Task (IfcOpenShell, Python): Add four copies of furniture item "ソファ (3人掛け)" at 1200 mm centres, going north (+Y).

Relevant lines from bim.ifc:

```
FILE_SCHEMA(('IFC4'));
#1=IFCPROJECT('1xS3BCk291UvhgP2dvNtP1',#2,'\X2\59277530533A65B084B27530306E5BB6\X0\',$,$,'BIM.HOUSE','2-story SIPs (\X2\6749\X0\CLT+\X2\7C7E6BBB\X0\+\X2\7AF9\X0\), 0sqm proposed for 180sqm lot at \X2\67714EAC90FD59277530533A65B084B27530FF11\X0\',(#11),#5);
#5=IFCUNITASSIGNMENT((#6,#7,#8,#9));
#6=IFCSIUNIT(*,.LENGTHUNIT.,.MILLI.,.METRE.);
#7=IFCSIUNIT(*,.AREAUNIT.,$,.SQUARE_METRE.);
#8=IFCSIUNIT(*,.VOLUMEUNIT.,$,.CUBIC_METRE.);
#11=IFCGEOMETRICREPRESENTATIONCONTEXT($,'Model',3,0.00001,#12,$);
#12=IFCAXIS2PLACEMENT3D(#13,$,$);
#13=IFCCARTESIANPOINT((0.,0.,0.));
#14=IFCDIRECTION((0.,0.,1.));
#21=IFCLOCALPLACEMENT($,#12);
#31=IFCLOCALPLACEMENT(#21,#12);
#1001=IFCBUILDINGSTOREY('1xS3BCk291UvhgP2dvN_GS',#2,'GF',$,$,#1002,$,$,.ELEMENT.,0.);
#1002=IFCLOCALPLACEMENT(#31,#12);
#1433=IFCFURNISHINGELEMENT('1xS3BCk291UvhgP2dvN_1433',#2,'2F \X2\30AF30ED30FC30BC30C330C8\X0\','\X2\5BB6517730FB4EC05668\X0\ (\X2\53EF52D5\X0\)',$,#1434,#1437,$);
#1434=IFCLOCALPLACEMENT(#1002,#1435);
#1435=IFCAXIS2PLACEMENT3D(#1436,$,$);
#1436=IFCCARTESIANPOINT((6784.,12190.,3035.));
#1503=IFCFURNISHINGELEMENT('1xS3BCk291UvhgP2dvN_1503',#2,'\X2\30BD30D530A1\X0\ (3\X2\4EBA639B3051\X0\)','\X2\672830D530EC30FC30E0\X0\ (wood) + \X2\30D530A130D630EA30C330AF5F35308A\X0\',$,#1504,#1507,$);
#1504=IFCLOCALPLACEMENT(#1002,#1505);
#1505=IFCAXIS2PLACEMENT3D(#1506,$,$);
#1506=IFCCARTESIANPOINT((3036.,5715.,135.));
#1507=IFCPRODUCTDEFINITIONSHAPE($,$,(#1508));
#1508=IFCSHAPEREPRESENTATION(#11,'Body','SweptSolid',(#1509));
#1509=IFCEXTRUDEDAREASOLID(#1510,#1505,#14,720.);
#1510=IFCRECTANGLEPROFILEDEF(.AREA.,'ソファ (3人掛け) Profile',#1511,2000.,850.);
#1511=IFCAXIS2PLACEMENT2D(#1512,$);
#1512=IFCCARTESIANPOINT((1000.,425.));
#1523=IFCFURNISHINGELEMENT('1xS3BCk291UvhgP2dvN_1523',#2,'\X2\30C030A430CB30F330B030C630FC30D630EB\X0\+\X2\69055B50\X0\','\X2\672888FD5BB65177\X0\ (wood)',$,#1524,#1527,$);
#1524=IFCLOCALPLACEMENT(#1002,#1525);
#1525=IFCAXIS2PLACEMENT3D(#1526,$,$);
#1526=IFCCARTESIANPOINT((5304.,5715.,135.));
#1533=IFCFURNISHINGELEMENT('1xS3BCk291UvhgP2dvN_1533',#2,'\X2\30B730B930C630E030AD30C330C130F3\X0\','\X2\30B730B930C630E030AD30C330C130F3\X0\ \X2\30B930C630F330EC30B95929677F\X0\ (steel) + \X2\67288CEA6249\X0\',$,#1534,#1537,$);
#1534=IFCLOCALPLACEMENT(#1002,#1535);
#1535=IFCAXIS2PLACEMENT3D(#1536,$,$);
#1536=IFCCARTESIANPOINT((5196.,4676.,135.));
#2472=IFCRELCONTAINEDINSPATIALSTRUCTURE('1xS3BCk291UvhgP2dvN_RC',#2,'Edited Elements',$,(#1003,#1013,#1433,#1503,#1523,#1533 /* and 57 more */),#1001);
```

```python
import numpy as np
import ifcopenshell
import ifcopenshell.api.geometry
import ifcopenshell.api.root
import ifcopenshell.util.element
import ifcopenshell.util.placement

model = ifcopenshell.open("bim.ifc")


def reuse_history(source, copy):
    """copy_class also copies each property set's owner history, people and application; keep the originals."""
    for rel in copy.IsDefinedBy:
        if rel.is_a("IfcRelDefinesByProperties") and (history := rel.RelatingPropertyDefinition.OwnerHistory):
            rel.RelatingPropertyDefinition.OwnerHistory = source.OwnerHistory
            ifcopenshell.util.element.remove_deep2(model, history)


source = model.by_id(1503)
base = ifcopenshell.util.placement.get_local_placement(source.ObjectPlacement)
step = np.array([0.0, 1.0, 0.0]) * 1200.0

for i in range(1, 5):
    copy = ifcopenshell.api.root.copy_class(model, product=source)
    copy.Representation = ifcopenshell.util.element.copy_deep(
        model, source.Representation, exclude=["IfcGeometricRepresentationContext", "IfcRepresentationMap"]
    )
    reuse_history(source, copy)
    matrix = base.copy()
    matrix[:3, 3] += i * step
    print("added at", matrix[:3, 3].round(3) + 0.0)
    ifcopenshell.api.geometry.edit_object_placement(model, product=copy, matrix=matrix, is_si=False)

model.write("bim-out.ifc")
```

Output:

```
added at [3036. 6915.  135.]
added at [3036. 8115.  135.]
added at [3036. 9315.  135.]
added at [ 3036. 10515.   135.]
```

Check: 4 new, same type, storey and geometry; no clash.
